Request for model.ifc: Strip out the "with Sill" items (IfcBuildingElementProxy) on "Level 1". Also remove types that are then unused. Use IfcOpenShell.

First a look at what the model holds.

```python
import ifcopenshell
import ifcopenshell.util.element

model = ifcopenshell.open("model.ifc")
print(model.schema)
storey = next(s for s in model.by_type("IfcBuildingStorey") if s.Name == "Level 1")
proxies = [e for e in ifcopenshell.util.element.get_decomposition(storey) if e.is_a("IfcBuildingElementProxy")]
seen = {}
for e in proxies:
    element_type = ifcopenshell.util.element.get_type(e)
    name = element_type.Name if element_type not in (None, e) else None
    seen[name] = seen.get(name, 0) + 1
for name, count in sorted(seen.items(), key=str):
    print(count, "x", name)
```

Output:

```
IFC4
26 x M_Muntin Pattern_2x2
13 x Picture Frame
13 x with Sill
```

```python
import ifcopenshell
import ifcopenshell.api.root
import ifcopenshell.util.element

model = ifcopenshell.open("model.ifc")

storey = next(s for s in model.by_type("IfcBuildingStorey") if s.Name == "Level 1")
proxies = [e for e in ifcopenshell.util.element.get_decomposition(storey) if e.is_a("IfcBuildingElementProxy")]
targets = [e for e in proxies if (t := ifcopenshell.util.element.get_type(e)) not in (None, e) and t.Name == "with Sill"]
types = {ifcopenshell.util.element.get_type(e) for e in targets} - {None, *targets}

for e in targets:
    ifcopenshell.api.root.remove_product(model, product=e)
print(len(targets), "removed")

unused = [t for t in types if not ifcopenshell.util.element.get_types(t)]
for t in unused:
    ifcopenshell.api.root.remove_product(model, product=t)
print(len(unused), "unused types removed")

model.write("model_edited.ifc")
```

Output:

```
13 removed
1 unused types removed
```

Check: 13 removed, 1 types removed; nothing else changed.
